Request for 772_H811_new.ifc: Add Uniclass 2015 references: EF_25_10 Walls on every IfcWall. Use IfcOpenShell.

First a look at what the model holds.

```python
import ifcopenshell

model = ifcopenshell.open("772_H811_new.ifc")
print(model.schema)
print("classifications:", [c.Name for c in model.by_type("IfcClassification")])
for ifc_class in ("IfcDoor", "IfcRoof", "IfcStair", "IfcWall", "IfcWindow"):
    print(ifc_class, len(model.by_type(ifc_class)))
```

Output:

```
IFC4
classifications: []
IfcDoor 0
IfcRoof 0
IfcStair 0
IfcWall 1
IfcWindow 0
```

```python
import ifcopenshell
import ifcopenshell.api.classification

model = ifcopenshell.open("772_H811_new.ifc")

system = ifcopenshell.api.classification.add_classification(model, classification="Uniclass 2015")

codes = {
    "IfcWall": ("EF_25_10", "Walls"),
}
for ifc_class, (code, name) in codes.items():
    products = model.by_type(ifc_class)
    ifcopenshell.api.classification.add_reference(
        model, products=products, classification=system, identification=code, name=name
    )
    print(code, len(products))

model.write("772_H811_new_rev.ifc")
```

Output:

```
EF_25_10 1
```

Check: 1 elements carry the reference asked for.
